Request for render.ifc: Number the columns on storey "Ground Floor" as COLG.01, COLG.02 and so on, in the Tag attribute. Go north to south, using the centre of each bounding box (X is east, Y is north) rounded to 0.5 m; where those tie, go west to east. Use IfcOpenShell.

First a look at what the model holds.

```python
import ifcopenshell
import ifcopenshell.util.element
import ifcopenshell.util.placement

model = ifcopenshell.open("render.ifc")
print(model.schema)
storey = next(s for s in model.by_type("IfcBuildingStorey") if s.Name == "Ground Floor")
columns = [e for e in ifcopenshell.util.element.get_decomposition(storey) if e.is_a("IfcColumn")]
for e in sorted(columns, key=lambda e: e.id()):
    origin = ifcopenshell.util.placement.get_local_placement(e.ObjectPlacement)[:3, 3]
    print(e.id(), e.Tag, e.Name, origin.round(2) + 0.0, sep=" | ")
```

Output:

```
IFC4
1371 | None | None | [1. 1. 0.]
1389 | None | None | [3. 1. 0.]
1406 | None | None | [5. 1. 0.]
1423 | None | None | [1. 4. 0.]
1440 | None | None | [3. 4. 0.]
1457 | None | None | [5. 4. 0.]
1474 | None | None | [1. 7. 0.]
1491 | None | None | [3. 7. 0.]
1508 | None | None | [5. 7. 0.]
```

```python
import ifcopenshell
import ifcopenshell.geom
import ifcopenshell.util.element
import ifcopenshell.util.shape

model = ifcopenshell.open("render.ifc")
settings = ifcopenshell.geom.settings()
settings.set("use-world-coords", True)


def centre(element):
    shape = ifcopenshell.geom.create_shape(settings, element)
    return ifcopenshell.util.shape.get_bbox_centroid(shape.geometry)


storey = next(s for s in model.by_type("IfcBuildingStorey") if s.Name == "Ground Floor")
columns = [e for e in ifcopenshell.util.element.get_decomposition(storey) if e.is_a("IfcColumn")]

# Insertion points can sit at a corner or the storey origin, so sort by the geometry (in metres).
centres = {e: centre(e) for e in columns}
columns.sort(key=lambda e: (-round(centres[e][1] / 0.5), centres[e][0]))

for i, e in enumerate(columns, start=1):
    number = f"COLG.{i:02d}"
    e.Tag = number
    print(e.id(), number)

model.write("render_rev.ifc")
```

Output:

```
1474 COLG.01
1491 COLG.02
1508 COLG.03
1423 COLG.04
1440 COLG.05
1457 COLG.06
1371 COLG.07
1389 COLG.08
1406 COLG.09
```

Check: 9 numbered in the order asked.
